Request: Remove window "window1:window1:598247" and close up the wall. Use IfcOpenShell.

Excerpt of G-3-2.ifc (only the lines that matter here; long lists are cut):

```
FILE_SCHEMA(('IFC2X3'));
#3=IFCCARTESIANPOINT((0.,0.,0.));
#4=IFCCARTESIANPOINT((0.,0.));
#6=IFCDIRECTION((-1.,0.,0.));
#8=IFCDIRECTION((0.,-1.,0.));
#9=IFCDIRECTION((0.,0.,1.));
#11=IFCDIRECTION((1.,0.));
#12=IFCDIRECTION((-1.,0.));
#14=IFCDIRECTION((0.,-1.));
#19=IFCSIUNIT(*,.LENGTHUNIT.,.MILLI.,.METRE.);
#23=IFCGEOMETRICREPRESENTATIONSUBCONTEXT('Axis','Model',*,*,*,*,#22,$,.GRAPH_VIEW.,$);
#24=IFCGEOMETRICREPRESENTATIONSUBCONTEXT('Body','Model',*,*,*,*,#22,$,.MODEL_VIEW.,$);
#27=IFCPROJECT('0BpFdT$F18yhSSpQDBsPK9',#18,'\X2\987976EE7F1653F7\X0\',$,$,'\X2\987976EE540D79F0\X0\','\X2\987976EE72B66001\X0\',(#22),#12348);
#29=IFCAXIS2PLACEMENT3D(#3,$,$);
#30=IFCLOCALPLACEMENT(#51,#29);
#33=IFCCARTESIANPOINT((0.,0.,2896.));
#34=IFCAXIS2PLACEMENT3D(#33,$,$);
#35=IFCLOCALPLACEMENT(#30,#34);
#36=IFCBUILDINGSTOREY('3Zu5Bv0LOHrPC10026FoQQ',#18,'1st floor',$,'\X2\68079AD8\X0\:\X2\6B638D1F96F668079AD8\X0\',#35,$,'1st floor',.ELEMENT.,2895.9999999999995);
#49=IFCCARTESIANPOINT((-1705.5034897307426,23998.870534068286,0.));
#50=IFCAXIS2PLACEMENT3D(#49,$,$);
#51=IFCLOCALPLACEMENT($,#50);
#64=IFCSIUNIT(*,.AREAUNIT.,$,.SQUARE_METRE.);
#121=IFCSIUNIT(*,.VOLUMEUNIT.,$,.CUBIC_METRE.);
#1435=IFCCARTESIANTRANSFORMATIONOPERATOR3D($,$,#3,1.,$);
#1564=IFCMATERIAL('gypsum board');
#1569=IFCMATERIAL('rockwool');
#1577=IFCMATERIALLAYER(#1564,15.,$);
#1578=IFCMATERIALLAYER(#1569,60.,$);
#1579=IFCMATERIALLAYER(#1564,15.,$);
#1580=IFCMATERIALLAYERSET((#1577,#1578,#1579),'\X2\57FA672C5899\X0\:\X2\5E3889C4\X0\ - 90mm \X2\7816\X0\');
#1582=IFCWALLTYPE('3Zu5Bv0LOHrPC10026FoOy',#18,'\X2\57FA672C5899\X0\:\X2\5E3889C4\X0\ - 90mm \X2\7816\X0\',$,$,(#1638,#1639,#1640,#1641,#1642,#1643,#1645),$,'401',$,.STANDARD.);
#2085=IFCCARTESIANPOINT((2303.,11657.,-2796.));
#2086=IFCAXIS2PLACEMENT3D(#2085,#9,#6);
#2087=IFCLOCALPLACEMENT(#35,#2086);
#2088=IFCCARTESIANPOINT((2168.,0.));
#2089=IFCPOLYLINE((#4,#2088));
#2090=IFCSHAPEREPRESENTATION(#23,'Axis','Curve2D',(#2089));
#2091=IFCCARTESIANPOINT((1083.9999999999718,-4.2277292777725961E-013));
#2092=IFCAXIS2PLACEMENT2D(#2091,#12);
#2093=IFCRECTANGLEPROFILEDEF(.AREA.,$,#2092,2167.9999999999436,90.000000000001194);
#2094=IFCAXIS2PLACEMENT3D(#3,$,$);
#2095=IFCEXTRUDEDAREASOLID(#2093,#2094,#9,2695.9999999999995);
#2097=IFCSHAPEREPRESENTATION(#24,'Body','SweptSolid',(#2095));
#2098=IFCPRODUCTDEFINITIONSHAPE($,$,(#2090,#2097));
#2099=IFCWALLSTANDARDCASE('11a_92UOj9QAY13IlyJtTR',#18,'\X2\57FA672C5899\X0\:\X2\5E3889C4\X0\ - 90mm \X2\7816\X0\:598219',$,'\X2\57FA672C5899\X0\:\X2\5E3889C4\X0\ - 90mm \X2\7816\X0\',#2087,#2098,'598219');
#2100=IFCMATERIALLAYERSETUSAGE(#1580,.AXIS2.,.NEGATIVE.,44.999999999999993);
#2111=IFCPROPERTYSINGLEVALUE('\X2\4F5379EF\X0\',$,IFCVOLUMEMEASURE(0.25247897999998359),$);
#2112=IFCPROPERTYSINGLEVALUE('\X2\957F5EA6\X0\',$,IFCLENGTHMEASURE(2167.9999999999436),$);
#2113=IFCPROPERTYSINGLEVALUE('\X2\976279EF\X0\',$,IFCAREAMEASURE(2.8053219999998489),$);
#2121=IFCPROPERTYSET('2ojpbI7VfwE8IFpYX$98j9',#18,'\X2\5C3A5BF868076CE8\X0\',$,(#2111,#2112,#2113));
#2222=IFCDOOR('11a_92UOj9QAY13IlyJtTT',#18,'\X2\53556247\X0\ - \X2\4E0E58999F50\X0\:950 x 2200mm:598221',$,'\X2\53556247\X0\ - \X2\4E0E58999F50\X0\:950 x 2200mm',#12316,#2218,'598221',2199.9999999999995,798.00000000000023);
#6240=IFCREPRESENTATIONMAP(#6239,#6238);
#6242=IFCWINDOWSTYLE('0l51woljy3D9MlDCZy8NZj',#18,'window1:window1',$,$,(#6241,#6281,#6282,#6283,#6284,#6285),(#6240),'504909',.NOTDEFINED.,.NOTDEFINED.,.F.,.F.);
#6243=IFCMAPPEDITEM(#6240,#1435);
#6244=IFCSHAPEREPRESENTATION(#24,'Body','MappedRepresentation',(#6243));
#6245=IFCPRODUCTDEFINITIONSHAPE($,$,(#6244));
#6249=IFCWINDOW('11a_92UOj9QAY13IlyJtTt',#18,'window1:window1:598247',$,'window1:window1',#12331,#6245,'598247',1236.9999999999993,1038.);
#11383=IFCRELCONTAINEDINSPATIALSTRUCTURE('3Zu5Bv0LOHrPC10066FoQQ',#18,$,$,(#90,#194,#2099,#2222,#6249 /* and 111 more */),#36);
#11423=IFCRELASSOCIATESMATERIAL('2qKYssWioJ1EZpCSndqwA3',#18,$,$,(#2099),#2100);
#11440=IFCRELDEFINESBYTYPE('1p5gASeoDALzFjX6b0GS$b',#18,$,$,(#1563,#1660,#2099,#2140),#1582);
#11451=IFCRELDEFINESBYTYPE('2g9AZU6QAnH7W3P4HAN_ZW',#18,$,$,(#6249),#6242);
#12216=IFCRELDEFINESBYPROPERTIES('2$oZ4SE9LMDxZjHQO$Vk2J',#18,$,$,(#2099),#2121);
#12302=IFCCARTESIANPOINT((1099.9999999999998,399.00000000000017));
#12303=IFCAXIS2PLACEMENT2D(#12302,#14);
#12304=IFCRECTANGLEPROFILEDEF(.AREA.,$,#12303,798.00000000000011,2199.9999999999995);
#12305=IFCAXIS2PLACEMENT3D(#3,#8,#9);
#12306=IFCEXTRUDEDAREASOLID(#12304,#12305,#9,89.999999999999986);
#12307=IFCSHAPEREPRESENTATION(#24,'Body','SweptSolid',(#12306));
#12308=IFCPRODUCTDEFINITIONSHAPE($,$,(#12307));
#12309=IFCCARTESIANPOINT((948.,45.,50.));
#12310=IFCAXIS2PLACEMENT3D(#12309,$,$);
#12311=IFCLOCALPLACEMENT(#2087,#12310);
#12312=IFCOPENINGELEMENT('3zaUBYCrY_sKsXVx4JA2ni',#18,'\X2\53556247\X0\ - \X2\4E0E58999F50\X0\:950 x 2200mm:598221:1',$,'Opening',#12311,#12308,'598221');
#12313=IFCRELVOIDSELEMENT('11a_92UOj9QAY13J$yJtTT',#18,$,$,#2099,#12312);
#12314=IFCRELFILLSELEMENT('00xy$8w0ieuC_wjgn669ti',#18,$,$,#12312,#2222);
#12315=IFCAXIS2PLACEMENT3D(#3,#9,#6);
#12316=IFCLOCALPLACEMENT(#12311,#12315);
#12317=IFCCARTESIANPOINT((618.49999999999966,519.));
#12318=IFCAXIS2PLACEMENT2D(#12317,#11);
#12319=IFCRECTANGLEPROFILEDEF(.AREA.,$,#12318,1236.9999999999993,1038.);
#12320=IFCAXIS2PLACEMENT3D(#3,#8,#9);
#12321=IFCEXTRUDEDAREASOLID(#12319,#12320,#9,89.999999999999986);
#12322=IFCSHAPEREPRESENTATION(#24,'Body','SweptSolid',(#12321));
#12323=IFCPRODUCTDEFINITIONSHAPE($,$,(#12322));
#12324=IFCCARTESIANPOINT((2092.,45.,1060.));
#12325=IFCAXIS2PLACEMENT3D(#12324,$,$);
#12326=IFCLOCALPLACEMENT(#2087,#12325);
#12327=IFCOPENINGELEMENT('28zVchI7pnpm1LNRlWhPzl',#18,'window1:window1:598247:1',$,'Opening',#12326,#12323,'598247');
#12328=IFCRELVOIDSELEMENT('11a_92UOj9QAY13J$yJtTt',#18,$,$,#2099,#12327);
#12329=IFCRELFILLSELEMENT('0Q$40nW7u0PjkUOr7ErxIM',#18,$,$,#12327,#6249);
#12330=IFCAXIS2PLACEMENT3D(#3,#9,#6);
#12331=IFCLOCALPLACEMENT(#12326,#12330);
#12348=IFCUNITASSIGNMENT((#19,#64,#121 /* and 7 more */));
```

```python
import ifcopenshell
import ifcopenshell.api.feature
import ifcopenshell.api.pset
import ifcopenshell.api.root
import ifcopenshell.geom
import ifcopenshell.util.element
import ifcopenshell.util.shape
import ifcopenshell.util.unit

model = ifcopenshell.open("G-3-2.ifc")
area_scale = ifcopenshell.util.unit.calculate_unit_scale(model, "AREAUNIT")
volume_scale = ifcopenshell.util.unit.calculate_unit_scale(model, "VOLUMEUNIT")
settings = ifcopenshell.geom.settings()


def volume(element):
    """Net volume in cubic metres, openings subtracted."""
    shape = ifcopenshell.geom.create_shape(settings, element)
    return ifcopenshell.util.shape.get_volume(shape.geometry)


window = model.by_guid("11a_92UOj9QAY13IlyJtTt")
opening = window.FillsVoids[0].RelatingOpeningElement
wall = opening.VoidsElements[0].RelatingBuildingElement
before = volume(wall)

ifcopenshell.api.root.remove_product(model, product=window)
ifcopenshell.api.feature.remove_feature(model, feature=opening)

after = volume(wall)
thickness = 0.09  # wall thickness in metres

# Update the wall's stored quantities.
pset = model.by_id(ifcopenshell.util.element.get_pset(wall, "尺寸标注", should_inherit=False)["id"])
ifcopenshell.api.pset.edit_pset(model, pset=pset, properties={
    "体积": model.create_entity("IfcVolumeMeasure", after / volume_scale),
    "面积": model.create_entity("IfcAreaMeasure", after / thickness / area_scale),
})

print(f"wall volume {before:.3f} -> {after:.3f} m3")

model.write("G-3-2_v2.ifc")
```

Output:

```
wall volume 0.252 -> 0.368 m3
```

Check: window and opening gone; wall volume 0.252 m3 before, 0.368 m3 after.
